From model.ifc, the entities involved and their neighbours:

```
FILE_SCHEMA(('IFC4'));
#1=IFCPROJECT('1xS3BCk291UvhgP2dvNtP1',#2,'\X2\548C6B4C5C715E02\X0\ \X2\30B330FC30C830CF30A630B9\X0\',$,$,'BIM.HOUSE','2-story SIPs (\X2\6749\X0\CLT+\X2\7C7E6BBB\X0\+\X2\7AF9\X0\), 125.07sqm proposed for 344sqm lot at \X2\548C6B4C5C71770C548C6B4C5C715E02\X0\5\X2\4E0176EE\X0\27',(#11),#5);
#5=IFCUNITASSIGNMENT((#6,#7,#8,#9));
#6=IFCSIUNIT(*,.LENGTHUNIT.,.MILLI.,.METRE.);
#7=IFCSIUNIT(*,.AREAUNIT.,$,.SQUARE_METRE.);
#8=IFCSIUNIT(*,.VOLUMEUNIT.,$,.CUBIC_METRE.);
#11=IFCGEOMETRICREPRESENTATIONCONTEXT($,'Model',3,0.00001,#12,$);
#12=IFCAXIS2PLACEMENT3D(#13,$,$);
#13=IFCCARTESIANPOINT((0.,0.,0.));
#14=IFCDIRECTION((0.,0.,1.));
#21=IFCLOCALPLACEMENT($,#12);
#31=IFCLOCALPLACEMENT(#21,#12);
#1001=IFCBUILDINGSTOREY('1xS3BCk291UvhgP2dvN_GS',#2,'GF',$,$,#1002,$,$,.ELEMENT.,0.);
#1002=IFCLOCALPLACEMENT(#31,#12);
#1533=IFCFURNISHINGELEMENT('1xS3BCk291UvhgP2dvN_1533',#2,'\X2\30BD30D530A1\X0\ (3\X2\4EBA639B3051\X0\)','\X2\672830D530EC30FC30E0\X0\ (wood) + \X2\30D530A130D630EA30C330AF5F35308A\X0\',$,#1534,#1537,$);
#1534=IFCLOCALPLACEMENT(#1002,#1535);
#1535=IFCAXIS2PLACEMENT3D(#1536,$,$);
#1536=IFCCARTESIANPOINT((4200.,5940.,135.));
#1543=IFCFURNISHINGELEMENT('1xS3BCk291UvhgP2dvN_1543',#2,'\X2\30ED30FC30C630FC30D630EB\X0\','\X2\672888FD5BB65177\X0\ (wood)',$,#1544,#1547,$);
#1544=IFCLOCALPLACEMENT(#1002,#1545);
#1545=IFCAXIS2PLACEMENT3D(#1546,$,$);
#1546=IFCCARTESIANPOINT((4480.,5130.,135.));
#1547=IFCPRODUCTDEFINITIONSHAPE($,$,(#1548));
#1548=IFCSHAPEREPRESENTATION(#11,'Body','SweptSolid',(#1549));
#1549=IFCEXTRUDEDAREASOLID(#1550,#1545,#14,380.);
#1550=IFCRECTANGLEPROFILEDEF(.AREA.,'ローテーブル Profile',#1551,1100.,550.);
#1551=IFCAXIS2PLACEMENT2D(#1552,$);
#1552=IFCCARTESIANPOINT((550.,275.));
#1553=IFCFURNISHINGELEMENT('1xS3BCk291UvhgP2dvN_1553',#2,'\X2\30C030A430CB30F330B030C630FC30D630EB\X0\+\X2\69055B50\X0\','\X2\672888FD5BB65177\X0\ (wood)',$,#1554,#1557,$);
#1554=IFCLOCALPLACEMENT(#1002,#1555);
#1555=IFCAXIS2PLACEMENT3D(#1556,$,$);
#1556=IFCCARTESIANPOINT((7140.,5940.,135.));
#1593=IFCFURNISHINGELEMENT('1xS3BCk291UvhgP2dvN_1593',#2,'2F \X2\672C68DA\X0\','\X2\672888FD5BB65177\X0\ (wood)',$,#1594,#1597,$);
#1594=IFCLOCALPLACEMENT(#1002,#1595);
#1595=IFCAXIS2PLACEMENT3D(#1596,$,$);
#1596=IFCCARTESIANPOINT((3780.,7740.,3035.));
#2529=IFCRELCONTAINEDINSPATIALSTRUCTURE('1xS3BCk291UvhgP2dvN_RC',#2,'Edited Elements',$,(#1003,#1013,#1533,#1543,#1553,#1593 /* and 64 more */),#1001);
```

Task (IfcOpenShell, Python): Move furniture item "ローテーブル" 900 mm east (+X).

```python
import ifcopenshell
import ifcopenshell.api.geometry
import ifcopenshell.util.placement
import ifcopenshell.util.unit

model = ifcopenshell.open("model.ifc")
unit_scale = ifcopenshell.util.unit.calculate_unit_scale(model)

item = model.by_guid("1xS3BCk291UvhgP2dvN_1543")
matrix = ifcopenshell.util.placement.get_local_placement(item.ObjectPlacement)
matrix[0, 3] += 0.9 / unit_scale
ifcopenshell.api.geometry.edit_object_placement(model, product=item, matrix=matrix, is_si=False)

print(ifcopenshell.util.placement.get_local_placement(item.ObjectPlacement).round(3) + 0.0)

model.write("model-out.ifc")
```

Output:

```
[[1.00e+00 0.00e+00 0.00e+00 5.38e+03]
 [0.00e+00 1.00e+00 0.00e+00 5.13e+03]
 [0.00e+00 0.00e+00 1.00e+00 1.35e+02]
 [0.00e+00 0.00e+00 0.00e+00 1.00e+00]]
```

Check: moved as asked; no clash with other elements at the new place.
